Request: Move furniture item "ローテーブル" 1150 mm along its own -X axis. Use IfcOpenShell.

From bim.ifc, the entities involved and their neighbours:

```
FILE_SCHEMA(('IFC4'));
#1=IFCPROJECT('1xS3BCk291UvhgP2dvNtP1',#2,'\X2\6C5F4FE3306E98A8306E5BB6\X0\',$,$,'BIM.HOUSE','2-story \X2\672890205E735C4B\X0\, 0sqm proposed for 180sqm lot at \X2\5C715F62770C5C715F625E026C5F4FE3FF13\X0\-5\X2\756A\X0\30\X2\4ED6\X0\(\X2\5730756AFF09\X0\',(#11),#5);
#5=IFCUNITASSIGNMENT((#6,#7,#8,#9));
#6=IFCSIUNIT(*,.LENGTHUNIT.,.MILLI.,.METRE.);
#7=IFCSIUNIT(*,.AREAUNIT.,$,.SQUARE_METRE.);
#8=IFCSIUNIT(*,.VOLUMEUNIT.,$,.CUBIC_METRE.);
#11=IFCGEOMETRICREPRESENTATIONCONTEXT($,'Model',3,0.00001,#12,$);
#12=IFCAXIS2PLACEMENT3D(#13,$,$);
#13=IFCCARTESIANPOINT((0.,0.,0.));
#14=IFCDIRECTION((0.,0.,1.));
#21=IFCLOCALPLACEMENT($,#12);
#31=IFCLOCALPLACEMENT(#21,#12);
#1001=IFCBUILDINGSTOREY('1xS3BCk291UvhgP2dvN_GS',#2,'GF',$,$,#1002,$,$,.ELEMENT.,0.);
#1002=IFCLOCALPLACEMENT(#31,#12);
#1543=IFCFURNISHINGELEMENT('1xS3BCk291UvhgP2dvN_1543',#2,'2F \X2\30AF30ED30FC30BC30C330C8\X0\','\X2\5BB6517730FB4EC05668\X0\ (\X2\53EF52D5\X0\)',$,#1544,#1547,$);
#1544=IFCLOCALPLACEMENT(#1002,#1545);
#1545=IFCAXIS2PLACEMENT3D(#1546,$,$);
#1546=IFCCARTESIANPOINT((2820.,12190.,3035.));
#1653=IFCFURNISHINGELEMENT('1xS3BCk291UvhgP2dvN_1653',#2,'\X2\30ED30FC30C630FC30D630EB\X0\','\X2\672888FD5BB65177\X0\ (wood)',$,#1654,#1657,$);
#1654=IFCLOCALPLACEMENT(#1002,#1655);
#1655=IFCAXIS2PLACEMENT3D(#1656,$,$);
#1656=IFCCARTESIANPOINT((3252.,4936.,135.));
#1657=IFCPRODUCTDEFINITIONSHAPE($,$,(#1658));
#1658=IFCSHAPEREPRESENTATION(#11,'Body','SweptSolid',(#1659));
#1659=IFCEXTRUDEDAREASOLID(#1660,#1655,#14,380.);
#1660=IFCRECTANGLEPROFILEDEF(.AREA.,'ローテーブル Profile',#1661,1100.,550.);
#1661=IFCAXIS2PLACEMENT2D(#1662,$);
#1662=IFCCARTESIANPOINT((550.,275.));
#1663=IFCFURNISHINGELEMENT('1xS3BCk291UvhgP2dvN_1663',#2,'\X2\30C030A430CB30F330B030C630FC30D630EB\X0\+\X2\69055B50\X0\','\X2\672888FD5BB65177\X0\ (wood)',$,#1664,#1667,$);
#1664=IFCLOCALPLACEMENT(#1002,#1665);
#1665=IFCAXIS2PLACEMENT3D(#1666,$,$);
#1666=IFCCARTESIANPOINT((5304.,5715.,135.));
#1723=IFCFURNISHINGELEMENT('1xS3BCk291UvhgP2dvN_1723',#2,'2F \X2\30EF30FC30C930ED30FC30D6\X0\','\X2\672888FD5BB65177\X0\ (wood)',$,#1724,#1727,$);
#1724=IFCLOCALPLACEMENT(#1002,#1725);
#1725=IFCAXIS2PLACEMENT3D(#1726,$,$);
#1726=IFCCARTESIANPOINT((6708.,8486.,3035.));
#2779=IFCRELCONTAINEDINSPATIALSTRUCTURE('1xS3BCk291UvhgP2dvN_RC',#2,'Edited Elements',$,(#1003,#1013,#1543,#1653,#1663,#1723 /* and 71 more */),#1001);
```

```python
import ifcopenshell
import ifcopenshell.api.geometry
import ifcopenshell.util.placement
import ifcopenshell.util.unit

model = ifcopenshell.open("bim.ifc")
unit_scale = ifcopenshell.util.unit.calculate_unit_scale(model)

item = model.by_id(1653)
matrix = ifcopenshell.util.placement.get_local_placement(item.ObjectPlacement)
matrix[:3, 3] -= matrix[:3, 0] * 1.15 / unit_scale
ifcopenshell.api.geometry.edit_object_placement(model, product=item, matrix=matrix, is_si=False)

print(ifcopenshell.util.placement.get_local_placement(item.ObjectPlacement).round(3) + 0.0)

model.write("bim_updated.ifc")
```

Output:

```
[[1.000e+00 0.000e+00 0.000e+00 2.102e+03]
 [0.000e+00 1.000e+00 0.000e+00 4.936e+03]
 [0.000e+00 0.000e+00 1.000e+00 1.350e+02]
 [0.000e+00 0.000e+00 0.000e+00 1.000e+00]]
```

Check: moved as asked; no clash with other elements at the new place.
